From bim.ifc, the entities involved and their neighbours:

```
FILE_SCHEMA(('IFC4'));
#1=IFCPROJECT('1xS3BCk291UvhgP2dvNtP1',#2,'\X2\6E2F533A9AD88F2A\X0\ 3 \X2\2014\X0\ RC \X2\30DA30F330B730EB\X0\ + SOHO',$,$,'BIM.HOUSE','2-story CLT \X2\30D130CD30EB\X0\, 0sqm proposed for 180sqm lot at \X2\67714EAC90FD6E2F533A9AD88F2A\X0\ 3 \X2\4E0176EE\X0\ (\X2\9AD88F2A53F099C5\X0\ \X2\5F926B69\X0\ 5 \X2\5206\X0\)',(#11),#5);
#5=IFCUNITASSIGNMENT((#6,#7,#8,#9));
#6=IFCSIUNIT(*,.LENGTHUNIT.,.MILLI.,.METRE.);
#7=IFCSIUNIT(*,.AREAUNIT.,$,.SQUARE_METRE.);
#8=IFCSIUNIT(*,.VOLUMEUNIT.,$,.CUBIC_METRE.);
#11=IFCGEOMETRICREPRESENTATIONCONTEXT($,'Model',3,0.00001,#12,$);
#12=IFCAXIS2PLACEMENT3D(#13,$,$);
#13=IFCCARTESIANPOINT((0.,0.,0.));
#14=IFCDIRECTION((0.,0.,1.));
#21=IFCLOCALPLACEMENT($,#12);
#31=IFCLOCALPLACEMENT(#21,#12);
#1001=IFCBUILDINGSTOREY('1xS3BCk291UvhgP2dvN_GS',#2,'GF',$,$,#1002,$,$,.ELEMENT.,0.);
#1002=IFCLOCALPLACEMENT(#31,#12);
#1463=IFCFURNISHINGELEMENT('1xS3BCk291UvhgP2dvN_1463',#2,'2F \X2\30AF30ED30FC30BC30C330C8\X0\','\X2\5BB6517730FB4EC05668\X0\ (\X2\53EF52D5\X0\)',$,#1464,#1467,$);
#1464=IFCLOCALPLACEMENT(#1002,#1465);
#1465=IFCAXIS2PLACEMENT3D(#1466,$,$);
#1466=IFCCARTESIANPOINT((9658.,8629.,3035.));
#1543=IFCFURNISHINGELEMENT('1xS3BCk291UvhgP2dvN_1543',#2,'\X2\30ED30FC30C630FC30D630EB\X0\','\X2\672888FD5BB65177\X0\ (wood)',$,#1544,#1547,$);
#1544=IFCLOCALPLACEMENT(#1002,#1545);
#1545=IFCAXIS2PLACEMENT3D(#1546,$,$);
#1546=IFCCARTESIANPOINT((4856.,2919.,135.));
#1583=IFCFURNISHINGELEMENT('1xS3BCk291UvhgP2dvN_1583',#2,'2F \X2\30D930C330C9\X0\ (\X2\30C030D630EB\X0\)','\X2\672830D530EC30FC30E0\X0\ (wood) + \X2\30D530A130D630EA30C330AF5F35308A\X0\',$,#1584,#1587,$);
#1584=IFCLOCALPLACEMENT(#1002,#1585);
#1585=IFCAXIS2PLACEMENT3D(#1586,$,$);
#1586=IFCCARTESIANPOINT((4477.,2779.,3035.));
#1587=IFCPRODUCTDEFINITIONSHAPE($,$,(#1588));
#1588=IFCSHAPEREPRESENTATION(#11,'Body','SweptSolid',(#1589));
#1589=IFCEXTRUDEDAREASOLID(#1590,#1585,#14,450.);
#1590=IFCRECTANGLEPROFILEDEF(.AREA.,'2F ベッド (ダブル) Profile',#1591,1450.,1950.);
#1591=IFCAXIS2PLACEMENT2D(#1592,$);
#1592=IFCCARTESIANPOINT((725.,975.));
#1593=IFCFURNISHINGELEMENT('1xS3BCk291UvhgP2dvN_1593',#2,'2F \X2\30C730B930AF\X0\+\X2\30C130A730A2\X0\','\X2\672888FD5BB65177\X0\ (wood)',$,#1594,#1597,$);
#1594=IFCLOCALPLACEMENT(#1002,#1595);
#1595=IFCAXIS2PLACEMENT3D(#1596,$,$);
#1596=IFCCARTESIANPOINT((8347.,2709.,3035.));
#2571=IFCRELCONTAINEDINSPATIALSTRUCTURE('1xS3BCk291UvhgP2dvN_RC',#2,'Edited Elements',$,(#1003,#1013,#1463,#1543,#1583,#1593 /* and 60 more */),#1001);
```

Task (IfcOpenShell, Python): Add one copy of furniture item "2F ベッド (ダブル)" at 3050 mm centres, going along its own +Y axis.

```python
import ifcopenshell
import ifcopenshell.api.geometry
import ifcopenshell.api.root
import ifcopenshell.util.element
import ifcopenshell.util.placement
import ifcopenshell.util.unit

model = ifcopenshell.open("bim.ifc")
unit_scale = ifcopenshell.util.unit.calculate_unit_scale(model)


def reuse_history(source, copy):
    """copy_class also copies each property set's owner history, people and application; keep the originals."""
    for rel in copy.IsDefinedBy:
        if rel.is_a("IfcRelDefinesByProperties") and (history := rel.RelatingPropertyDefinition.OwnerHistory):
            rel.RelatingPropertyDefinition.OwnerHistory = source.OwnerHistory
            ifcopenshell.util.element.remove_deep2(model, history)


source = model.by_id(1583)
base = ifcopenshell.util.placement.get_local_placement(source.ObjectPlacement)
step = base[:3, 1] * 3.05 / unit_scale

for i in range(1, 2):
    copy = ifcopenshell.api.root.copy_class(model, product=source)
    copy.Representation = ifcopenshell.util.element.copy_deep(
        model, source.Representation, exclude=["IfcGeometricRepresentationContext", "IfcRepresentationMap"]
    )
    reuse_history(source, copy)
    matrix = base.copy()
    matrix[:3, 3] += i * step
    print("added at", matrix[:3, 3].round(3) + 0.0)
    ifcopenshell.api.geometry.edit_object_placement(model, product=copy, matrix=matrix, is_si=False)

model.write("bim-out.ifc")
```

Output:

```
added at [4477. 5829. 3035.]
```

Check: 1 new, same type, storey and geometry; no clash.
